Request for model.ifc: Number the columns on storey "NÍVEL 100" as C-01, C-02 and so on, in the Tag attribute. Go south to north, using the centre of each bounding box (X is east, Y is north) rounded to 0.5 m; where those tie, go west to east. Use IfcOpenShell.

First a look at what the model holds.

```python
import ifcopenshell
import ifcopenshell.util.element
import ifcopenshell.util.placement

model = ifcopenshell.open("model.ifc")
print(model.schema)
storey = next(s for s in model.by_type("IfcBuildingStorey") if s.Name == "NÍVEL 100")
columns = [e for e in ifcopenshell.util.element.get_decomposition(storey) if e.is_a("IfcColumn")]
for e in sorted(columns, key=lambda e: e.id()):
    origin = ifcopenshell.util.placement.get_local_placement(e.ObjectPlacement)[:3, 3]
    print(e.id(), e.Tag, e.Name, origin.round(2) + 0.0, sep=" | ")
```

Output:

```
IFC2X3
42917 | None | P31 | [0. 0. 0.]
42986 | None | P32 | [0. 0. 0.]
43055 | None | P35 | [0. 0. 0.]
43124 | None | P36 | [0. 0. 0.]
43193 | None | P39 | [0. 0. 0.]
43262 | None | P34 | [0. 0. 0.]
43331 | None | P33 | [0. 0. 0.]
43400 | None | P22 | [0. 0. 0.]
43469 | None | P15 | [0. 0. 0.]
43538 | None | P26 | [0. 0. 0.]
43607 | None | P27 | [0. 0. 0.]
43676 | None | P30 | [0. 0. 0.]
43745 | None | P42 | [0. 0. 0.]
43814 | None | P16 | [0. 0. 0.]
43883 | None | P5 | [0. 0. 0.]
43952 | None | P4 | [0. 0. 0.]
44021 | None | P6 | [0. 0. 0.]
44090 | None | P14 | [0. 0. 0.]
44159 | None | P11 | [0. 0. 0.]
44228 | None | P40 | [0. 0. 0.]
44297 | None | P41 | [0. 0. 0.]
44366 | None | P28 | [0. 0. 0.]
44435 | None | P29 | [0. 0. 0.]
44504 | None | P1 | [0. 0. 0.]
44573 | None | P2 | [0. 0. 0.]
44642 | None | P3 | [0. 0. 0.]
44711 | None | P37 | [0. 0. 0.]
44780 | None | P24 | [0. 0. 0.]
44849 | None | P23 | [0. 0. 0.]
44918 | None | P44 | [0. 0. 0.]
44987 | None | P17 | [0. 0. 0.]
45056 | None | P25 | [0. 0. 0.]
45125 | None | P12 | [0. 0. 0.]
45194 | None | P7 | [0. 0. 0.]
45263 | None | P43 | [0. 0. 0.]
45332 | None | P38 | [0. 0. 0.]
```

```python
import ifcopenshell
import ifcopenshell.geom
import ifcopenshell.util.element
import ifcopenshell.util.shape

model = ifcopenshell.open("model.ifc")
settings = ifcopenshell.geom.settings()
settings.set("use-world-coords", True)


def centre(element):
    shape = ifcopenshell.geom.create_shape(settings, element)
    return ifcopenshell.util.shape.get_bbox_centroid(shape.geometry)


storey = next(s for s in model.by_type("IfcBuildingStorey") if s.Name == "NÍVEL 100")
columns = [e for e in ifcopenshell.util.element.get_decomposition(storey) if e.is_a("IfcColumn")]

# Insertion points can sit at a corner or the storey origin, so sort by the geometry (in metres).
centres = {e: centre(e) for e in columns}
columns.sort(key=lambda e: (round(centres[e][1] / 0.5), centres[e][0]))

for i, e in enumerate(columns, start=1):
    number = f"C-{i:02d}"
    e.Tag = number
    print(e.id(), number)

model.write("model_v2.ifc")
```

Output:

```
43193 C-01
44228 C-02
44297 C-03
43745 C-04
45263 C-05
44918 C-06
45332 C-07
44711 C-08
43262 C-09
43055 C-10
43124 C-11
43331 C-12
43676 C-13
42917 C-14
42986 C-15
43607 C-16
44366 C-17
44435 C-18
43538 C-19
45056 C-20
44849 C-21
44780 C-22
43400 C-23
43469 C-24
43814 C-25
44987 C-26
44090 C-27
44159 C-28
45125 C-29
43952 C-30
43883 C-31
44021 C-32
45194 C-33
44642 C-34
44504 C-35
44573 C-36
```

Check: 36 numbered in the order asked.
